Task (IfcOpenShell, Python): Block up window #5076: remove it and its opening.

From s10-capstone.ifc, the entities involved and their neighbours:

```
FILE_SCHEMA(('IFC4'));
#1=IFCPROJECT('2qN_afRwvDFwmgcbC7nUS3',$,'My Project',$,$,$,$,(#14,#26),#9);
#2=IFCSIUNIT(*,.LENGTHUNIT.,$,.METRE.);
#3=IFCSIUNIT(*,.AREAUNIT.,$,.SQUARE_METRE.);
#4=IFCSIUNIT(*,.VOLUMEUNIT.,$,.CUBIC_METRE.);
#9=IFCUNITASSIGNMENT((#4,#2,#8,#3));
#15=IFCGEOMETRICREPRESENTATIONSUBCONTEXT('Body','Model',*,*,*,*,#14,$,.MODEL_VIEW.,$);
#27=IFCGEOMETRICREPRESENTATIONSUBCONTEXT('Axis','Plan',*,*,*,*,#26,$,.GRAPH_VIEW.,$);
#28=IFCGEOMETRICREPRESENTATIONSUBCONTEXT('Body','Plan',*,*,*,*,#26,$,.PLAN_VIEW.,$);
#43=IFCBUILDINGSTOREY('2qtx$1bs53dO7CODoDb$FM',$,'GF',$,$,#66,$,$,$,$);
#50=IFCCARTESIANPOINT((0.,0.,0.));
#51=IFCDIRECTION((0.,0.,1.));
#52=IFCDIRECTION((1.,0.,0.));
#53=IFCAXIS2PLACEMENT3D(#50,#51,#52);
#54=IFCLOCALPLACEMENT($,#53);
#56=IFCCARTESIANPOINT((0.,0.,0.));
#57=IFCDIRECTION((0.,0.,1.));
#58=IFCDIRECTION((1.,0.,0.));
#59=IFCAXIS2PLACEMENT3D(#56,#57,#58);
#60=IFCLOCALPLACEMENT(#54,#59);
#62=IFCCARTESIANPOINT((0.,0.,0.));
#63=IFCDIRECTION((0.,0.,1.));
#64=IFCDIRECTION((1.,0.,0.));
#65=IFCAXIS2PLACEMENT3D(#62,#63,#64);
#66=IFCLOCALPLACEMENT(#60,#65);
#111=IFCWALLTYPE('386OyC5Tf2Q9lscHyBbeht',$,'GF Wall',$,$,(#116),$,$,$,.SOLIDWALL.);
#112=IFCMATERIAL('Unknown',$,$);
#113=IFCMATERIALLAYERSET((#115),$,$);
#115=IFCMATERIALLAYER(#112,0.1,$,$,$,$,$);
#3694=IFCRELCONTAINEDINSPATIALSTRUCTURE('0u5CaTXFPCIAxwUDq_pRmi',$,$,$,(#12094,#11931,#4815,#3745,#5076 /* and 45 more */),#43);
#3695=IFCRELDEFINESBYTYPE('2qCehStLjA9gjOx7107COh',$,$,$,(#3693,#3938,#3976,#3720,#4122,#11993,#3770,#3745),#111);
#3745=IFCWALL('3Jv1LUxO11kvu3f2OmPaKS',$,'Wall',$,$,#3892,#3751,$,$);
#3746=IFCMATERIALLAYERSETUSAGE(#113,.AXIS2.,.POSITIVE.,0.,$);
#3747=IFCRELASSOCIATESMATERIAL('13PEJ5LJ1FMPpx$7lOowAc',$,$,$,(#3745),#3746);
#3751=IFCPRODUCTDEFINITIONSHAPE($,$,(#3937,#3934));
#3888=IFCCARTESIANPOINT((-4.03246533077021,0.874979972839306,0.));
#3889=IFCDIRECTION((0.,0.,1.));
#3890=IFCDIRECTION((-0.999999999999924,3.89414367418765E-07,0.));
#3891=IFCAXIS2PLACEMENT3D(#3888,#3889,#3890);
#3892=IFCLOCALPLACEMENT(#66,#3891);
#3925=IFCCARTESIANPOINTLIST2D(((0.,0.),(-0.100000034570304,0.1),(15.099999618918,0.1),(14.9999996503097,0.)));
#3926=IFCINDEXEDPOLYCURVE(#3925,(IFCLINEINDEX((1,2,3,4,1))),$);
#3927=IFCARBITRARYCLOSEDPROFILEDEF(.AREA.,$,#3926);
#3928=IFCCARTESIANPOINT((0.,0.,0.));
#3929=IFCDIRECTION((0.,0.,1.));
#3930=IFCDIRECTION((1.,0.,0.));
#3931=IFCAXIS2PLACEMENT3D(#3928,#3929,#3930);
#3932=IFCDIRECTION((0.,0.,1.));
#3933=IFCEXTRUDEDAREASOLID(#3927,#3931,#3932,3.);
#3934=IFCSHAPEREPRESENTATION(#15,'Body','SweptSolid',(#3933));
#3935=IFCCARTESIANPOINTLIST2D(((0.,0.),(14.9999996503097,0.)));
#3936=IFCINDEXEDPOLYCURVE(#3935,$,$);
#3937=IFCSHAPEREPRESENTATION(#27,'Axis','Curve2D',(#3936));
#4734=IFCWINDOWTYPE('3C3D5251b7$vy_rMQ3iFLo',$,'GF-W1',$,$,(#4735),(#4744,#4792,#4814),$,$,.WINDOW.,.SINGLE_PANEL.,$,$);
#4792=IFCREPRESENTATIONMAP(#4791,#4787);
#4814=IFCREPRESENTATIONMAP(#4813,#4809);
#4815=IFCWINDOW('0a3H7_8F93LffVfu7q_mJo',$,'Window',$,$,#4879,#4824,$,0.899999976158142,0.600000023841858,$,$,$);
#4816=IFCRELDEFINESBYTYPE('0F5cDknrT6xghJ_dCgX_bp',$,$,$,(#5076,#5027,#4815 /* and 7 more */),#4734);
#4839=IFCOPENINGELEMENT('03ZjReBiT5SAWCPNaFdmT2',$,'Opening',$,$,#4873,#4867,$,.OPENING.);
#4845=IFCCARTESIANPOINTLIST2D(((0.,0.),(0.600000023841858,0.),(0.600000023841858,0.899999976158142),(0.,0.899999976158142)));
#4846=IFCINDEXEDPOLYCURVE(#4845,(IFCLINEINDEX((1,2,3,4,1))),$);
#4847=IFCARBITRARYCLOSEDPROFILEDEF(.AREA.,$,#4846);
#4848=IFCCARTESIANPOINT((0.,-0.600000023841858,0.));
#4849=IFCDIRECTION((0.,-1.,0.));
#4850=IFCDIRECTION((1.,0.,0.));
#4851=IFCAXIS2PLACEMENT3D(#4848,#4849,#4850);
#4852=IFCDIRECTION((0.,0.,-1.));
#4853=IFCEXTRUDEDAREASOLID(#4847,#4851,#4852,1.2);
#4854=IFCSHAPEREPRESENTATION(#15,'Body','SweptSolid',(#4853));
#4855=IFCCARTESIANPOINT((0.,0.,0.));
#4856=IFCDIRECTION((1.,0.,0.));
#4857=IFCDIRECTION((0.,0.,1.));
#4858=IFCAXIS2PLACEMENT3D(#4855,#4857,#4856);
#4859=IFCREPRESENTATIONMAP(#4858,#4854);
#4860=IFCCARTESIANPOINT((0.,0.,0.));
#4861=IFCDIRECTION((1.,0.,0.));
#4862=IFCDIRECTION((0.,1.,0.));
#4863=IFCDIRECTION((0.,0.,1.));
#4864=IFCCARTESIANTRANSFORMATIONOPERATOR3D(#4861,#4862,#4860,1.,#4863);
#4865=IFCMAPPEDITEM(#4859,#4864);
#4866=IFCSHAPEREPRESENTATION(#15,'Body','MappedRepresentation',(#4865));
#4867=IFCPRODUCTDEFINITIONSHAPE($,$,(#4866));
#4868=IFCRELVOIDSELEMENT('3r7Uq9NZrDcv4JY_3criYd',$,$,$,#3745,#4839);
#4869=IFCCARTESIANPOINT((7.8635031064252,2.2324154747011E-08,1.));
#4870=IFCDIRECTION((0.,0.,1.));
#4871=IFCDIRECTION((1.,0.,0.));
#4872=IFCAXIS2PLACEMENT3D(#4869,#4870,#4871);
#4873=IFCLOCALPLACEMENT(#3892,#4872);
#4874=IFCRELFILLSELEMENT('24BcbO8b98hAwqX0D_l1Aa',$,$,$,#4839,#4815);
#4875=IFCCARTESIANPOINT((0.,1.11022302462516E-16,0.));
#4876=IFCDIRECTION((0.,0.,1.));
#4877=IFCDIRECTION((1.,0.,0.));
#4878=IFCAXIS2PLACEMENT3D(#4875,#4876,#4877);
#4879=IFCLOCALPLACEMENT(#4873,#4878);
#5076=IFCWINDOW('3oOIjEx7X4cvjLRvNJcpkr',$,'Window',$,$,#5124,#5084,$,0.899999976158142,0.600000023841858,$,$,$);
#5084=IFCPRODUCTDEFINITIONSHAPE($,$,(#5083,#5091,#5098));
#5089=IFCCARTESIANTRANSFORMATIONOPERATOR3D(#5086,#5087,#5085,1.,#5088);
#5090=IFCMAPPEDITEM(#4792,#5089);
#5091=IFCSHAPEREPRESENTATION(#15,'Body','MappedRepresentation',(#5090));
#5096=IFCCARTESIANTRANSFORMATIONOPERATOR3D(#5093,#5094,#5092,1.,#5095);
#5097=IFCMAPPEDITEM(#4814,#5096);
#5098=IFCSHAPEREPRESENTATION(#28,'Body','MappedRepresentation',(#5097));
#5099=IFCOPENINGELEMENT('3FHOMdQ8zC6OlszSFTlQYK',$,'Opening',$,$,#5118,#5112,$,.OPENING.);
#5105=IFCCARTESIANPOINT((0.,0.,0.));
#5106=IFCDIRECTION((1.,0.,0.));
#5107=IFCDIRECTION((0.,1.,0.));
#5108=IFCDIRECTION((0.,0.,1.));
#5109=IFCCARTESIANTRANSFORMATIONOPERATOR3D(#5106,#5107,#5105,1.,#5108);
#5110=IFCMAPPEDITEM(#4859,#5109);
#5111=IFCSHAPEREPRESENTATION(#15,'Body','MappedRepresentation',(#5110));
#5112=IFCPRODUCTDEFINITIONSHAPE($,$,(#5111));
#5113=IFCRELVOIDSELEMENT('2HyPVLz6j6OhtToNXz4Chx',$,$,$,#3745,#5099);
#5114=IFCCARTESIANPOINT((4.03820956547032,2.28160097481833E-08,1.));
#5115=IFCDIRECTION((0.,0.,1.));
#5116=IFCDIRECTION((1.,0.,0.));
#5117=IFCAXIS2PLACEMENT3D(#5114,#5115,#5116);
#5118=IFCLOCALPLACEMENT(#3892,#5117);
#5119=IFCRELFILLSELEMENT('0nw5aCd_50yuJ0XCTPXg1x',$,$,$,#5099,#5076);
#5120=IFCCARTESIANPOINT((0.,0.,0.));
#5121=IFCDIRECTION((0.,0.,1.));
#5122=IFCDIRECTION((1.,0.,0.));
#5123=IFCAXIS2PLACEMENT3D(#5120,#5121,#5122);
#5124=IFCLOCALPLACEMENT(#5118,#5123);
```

```python
import ifcopenshell
import ifcopenshell.api.feature
import ifcopenshell.api.root
import ifcopenshell.geom
import ifcopenshell.util.shape

model = ifcopenshell.open("s10-capstone.ifc")
settings = ifcopenshell.geom.settings()


def volume(element):
    """Net volume in cubic metres, openings subtracted."""
    shape = ifcopenshell.geom.create_shape(settings, element)
    return ifcopenshell.util.shape.get_volume(shape.geometry)


window = model.by_guid("3oOIjEx7X4cvjLRvNJcpkr")
opening = window.FillsVoids[0].RelatingOpeningElement
wall = opening.VoidsElements[0].RelatingBuildingElement
before = volume(wall)

ifcopenshell.api.root.remove_product(model, product=window)
ifcopenshell.api.feature.remove_feature(model, feature=opening)

after = volume(wall)

print(f"wall volume {before:.3f} -> {after:.3f} m3")

model.write("s10-capstone_edited.ifc")
```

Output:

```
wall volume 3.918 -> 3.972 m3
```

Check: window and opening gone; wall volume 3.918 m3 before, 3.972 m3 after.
